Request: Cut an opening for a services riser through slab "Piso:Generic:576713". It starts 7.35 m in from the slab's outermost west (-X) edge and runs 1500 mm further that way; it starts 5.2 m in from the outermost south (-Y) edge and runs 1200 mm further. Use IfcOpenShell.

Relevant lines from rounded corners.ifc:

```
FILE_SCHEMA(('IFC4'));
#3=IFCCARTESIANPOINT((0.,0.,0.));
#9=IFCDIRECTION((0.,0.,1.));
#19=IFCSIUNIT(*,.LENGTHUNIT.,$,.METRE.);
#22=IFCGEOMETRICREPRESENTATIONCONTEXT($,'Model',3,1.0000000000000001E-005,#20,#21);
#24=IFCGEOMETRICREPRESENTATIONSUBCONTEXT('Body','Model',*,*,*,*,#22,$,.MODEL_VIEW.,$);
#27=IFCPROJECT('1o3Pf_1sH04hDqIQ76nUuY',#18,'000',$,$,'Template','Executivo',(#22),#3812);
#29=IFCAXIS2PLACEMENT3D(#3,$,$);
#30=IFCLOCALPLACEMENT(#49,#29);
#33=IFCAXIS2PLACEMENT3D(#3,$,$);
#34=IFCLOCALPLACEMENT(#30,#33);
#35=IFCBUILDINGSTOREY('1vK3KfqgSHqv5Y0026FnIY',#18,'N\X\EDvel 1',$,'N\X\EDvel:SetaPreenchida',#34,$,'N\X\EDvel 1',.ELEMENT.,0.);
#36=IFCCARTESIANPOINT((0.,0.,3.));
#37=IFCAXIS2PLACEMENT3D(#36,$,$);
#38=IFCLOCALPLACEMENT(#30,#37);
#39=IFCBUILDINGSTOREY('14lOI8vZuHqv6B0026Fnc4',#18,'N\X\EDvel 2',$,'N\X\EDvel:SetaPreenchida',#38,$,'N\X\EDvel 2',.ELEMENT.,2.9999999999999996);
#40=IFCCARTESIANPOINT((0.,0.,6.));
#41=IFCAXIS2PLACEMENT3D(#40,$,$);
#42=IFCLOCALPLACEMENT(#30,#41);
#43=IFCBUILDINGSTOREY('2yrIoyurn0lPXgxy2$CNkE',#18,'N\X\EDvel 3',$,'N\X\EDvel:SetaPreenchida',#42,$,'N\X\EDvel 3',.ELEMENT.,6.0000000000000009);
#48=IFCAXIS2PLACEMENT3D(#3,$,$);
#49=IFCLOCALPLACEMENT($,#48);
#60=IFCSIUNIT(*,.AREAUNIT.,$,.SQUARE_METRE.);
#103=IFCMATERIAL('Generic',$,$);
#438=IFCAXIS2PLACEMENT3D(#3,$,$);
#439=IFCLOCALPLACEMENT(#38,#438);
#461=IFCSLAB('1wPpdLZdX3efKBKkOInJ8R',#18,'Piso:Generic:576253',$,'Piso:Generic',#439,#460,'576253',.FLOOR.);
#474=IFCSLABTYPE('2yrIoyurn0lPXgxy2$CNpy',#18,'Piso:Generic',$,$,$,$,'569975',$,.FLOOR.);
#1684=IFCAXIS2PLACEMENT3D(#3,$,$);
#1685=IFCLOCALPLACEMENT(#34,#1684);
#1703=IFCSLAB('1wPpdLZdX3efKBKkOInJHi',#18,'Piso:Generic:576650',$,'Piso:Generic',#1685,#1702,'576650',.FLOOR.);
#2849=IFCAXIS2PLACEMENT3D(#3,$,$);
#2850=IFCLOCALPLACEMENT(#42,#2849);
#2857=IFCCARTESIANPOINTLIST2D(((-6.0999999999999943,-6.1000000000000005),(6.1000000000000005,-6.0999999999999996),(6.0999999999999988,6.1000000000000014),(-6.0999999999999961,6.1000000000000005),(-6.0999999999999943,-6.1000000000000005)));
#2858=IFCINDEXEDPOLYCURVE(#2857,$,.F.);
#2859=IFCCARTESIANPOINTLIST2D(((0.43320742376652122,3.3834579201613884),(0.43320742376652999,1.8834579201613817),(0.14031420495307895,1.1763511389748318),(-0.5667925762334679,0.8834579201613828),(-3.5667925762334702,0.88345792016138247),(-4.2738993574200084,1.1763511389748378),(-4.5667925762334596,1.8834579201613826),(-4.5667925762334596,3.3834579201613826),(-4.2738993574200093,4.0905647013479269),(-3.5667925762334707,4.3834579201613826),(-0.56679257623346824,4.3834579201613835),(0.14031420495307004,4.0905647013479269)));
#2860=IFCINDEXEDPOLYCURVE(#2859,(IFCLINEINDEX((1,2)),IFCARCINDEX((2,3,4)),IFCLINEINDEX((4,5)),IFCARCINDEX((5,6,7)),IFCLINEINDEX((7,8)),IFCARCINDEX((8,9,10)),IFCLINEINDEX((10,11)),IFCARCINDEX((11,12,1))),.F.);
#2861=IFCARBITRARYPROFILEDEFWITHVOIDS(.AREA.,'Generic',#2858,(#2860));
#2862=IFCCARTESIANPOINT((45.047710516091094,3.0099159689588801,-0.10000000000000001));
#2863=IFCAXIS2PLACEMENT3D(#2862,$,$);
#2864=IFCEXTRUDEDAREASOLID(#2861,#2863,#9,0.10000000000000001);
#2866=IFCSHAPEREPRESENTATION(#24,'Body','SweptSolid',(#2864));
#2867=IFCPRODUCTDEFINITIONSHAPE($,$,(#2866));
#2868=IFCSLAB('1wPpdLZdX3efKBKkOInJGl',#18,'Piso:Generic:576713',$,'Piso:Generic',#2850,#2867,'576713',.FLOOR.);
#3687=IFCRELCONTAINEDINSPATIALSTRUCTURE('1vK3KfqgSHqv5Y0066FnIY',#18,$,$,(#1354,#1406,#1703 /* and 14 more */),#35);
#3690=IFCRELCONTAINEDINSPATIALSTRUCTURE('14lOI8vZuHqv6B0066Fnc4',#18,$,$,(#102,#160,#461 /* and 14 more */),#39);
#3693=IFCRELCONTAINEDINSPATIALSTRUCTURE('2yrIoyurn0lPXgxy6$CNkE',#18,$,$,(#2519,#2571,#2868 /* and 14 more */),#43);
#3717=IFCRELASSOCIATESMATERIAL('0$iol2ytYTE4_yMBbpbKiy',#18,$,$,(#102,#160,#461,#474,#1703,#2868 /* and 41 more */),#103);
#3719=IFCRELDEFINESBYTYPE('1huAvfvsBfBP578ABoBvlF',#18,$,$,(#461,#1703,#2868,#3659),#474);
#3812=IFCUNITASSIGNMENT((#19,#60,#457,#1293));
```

```python
import numpy as np
import ifcopenshell
import ifcopenshell.api.feature
import ifcopenshell.api.geometry
import ifcopenshell.api.root
import ifcopenshell.geom
import ifcopenshell.util.placement
import ifcopenshell.util.representation
import ifcopenshell.util.shape
import ifcopenshell.util.unit

model = ifcopenshell.open("rounded corners.ifc")
unit_scale = ifcopenshell.util.unit.calculate_unit_scale(model)
settings = ifcopenshell.geom.settings()


def volume(element):
    """Net volume in cubic metres, openings subtracted."""
    shape = ifcopenshell.geom.create_shape(settings, element)
    return ifcopenshell.util.shape.get_volume(shape.geometry)


slab = model.by_id(2868)
before = volume(slab)

# Extent in the slab's own axes, in metres. The edges named are its -X and -Y sides.
slab_shape = ifcopenshell.geom.create_shape(settings, slab)
vertices = ifcopenshell.util.shape.get_vertices(slab_shape.geometry)
x_min, y_min, bottom = vertices.min(axis=0)
top = vertices[:, 2].max()

opening = ifcopenshell.api.root.create_entity(model, ifc_class="IfcOpeningElement", name="Services riser opening", predefined_type="OPENING")
context = ifcopenshell.util.representation.get_context(model, "Model", "Body", "MODEL_VIEW")
width, depth = 1.5, 1.2
outline = [(0.0, 0.0), (width, 0.0), (width, depth), (0.0, depth), (0.0, 0.0)]
# Overshoot both faces by 50 mm so the cut is clean.
shape = ifcopenshell.api.geometry.add_slab_representation(
    model, context=context, depth=top - bottom + 0.1, polyline=outline
)
ifcopenshell.api.geometry.assign_representation(model, product=opening, representation=shape)

matrix = ifcopenshell.util.placement.get_local_placement(slab.ObjectPlacement)
matrix[:, 3] = matrix @ np.append(np.array([x_min + 7.35, y_min + 5.2, bottom - 0.05]) / unit_scale, 1.0)
ifcopenshell.api.geometry.edit_object_placement(model, product=opening, matrix=matrix, is_si=False)
ifcopenshell.api.feature.add_feature(model, feature=opening, element=slab)

after = volume(slab)

print(f"slab volume {before:.3f} -> {after:.3f} m3")

model.write("rounded corners_edited.ifc")
```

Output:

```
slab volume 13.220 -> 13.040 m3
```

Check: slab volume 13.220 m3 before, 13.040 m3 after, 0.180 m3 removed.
